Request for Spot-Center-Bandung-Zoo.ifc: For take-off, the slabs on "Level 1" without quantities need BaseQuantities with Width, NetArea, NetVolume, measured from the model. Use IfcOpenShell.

First a look at what the model holds.

```python
import ifcopenshell
import ifcopenshell.util.element
import ifcopenshell.util.unit

model = ifcopenshell.open("Spot-Center-Bandung-Zoo.ifc")
print(model.schema)
for unit_type in ("LENGTHUNIT", "AREAUNIT", "VOLUMEUNIT"):
    print(unit_type, ifcopenshell.util.unit.calculate_unit_scale(model, unit_type))
storey = next(s for s in model.by_type("IfcBuildingStorey") if s.Name == "Level 1")
slabs = [e for e in ifcopenshell.util.element.get_decomposition(storey) if e.is_a("IfcSlab")]
for e in sorted(slabs, key=lambda e: e.id()):
    print(e.id(), e.is_a(), e.Name, list(ifcopenshell.util.element.get_psets(e, qtos_only=True)), sep=" | ")
```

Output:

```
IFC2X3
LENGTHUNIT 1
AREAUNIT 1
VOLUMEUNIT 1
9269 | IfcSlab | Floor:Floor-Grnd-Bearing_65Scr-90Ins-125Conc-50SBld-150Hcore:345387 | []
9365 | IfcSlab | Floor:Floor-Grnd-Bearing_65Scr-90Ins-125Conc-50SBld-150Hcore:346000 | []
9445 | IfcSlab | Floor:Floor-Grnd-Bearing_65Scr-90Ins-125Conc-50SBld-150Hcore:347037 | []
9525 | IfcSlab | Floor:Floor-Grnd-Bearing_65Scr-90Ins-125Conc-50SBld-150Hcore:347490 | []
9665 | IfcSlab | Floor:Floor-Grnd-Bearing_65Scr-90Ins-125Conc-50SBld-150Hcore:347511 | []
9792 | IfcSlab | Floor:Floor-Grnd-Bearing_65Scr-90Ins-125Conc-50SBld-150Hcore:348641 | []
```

```python
import ifcopenshell
import ifcopenshell.api.pset
import ifcopenshell.geom
import ifcopenshell.util.element
import ifcopenshell.util.shape
import ifcopenshell.util.unit

model = ifcopenshell.open("Spot-Center-Bandung-Zoo.ifc")
unit_scale = ifcopenshell.util.unit.calculate_unit_scale(model)
area_scale = ifcopenshell.util.unit.calculate_unit_scale(model, "AREAUNIT")
volume_scale = ifcopenshell.util.unit.calculate_unit_scale(model, "VOLUMEUNIT")
settings = ifcopenshell.geom.settings()

storey = next(s for s in model.by_type("IfcBuildingStorey") if s.Name == "Level 1")
slabs = [e for e in ifcopenshell.util.element.get_decomposition(storey) if e.is_a("IfcSlab")]

for e in sorted(slabs, key=lambda e: e.id()):
    if ifcopenshell.util.element.get_psets(e, qtos_only=True, should_inherit=False):
        continue
    # Geometry comes back in metres, in the element's own axes.
    shape = ifcopenshell.geom.create_shape(settings, e)
    values = {
        "Width": ifcopenshell.util.shape.get_z(shape.geometry) / unit_scale,
        "NetArea": ifcopenshell.util.shape.get_footprint_area(shape.geometry) / area_scale,
        "NetVolume": ifcopenshell.util.shape.get_volume(shape.geometry) / volume_scale,
    }
    qto = ifcopenshell.api.pset.add_qto(model, product=e, name="BaseQuantities")
    ifcopenshell.api.pset.edit_qto(model, qto=qto, properties=values)
    print(e.id(), {k: round(v, 3) for k, v in values.items()})

model.write("Spot-Center-Bandung-Zoo_v2.ifc")
```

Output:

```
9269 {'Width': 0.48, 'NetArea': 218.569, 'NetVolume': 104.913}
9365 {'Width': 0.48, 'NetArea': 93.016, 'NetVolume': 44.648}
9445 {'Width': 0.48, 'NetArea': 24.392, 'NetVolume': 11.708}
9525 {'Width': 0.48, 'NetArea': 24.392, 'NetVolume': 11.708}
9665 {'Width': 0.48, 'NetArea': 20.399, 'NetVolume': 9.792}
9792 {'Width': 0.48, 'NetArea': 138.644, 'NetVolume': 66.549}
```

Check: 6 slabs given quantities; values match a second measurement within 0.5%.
